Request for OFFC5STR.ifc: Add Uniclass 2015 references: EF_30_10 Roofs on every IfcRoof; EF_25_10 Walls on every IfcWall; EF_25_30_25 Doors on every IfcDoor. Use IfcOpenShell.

First a look at what the model holds.

```python
import ifcopenshell

model = ifcopenshell.open("OFFC5STR.ifc")
print(model.schema)
print("classifications:", [c.Name for c in model.by_type("IfcClassification")])
for ifc_class in ("IfcDoor", "IfcRoof", "IfcStair", "IfcWall", "IfcWindow"):
    print(ifc_class, len(model.by_type(ifc_class)))
```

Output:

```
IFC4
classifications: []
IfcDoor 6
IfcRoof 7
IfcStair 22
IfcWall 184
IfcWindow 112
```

```python
import ifcopenshell
import ifcopenshell.api.classification

model = ifcopenshell.open("OFFC5STR.ifc")

system = ifcopenshell.api.classification.add_classification(model, classification="Uniclass 2015")

codes = {
    "IfcRoof": ("EF_30_10", "Roofs"),
    "IfcWall": ("EF_25_10", "Walls"),
    "IfcDoor": ("EF_25_30_25", "Doors"),
}
for ifc_class, (code, name) in codes.items():
    products = model.by_type(ifc_class)
    ifcopenshell.api.classification.add_reference(
        model, products=products, classification=system, identification=code, name=name
    )
    print(code, len(products))

model.write("OFFC5STR-out.ifc")
```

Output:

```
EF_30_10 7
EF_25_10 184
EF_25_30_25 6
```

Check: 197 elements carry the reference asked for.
